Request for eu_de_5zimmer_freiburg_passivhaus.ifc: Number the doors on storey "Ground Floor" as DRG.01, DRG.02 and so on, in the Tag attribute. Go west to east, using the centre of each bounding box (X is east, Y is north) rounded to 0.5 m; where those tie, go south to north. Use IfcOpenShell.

First a look at what the model holds.

```python
import ifcopenshell
import ifcopenshell.util.element
import ifcopenshell.util.placement

model = ifcopenshell.open("eu_de_5zimmer_freiburg_passivhaus.ifc")
print(model.schema)
storey = next(s for s in model.by_type("IfcBuildingStorey") if s.Name == "Ground Floor")
doors = [e for e in ifcopenshell.util.element.get_decomposition(storey) if e.is_a("IfcDoor")]
for e in sorted(doors, key=lambda e: e.id()):
    origin = ifcopenshell.util.placement.get_local_placement(e.ObjectPlacement)[:3, 3]
    print(e.id(), e.Tag, e.Name, origin.round(2) + 0.0, sep=" | ")
```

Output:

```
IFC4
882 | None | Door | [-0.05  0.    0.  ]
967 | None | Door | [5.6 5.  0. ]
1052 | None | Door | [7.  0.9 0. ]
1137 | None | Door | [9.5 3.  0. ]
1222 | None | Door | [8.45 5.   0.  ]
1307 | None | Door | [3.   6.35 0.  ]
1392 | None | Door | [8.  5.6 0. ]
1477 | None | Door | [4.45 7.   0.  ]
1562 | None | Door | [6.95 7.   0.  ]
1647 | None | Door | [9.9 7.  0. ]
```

```python
import ifcopenshell
import ifcopenshell.geom
import ifcopenshell.util.element
import ifcopenshell.util.shape

model = ifcopenshell.open("eu_de_5zimmer_freiburg_passivhaus.ifc")
settings = ifcopenshell.geom.settings()
settings.set("use-world-coords", True)


def centre(element):
    shape = ifcopenshell.geom.create_shape(settings, element)
    return ifcopenshell.util.shape.get_bbox_centroid(shape.geometry)


storey = next(s for s in model.by_type("IfcBuildingStorey") if s.Name == "Ground Floor")
doors = [e for e in ifcopenshell.util.element.get_decomposition(storey) if e.is_a("IfcDoor")]

# Insertion points can sit at a corner or the storey origin, so sort by the geometry (in metres).
centres = {e: centre(e) for e in doors}
doors.sort(key=lambda e: (round(centres[e][0] / 0.5), centres[e][1]))

for i, e in enumerate(doors, start=1):
    number = f"DRG.{i:02d}"
    e.Tag = number
    print(e.id(), number)

model.write("eu_de_5zimmer_freiburg_passivhaus_v2.ifc")
```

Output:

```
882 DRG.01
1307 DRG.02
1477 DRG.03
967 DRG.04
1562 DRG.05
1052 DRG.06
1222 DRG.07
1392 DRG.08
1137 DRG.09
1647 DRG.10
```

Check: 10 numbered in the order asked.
